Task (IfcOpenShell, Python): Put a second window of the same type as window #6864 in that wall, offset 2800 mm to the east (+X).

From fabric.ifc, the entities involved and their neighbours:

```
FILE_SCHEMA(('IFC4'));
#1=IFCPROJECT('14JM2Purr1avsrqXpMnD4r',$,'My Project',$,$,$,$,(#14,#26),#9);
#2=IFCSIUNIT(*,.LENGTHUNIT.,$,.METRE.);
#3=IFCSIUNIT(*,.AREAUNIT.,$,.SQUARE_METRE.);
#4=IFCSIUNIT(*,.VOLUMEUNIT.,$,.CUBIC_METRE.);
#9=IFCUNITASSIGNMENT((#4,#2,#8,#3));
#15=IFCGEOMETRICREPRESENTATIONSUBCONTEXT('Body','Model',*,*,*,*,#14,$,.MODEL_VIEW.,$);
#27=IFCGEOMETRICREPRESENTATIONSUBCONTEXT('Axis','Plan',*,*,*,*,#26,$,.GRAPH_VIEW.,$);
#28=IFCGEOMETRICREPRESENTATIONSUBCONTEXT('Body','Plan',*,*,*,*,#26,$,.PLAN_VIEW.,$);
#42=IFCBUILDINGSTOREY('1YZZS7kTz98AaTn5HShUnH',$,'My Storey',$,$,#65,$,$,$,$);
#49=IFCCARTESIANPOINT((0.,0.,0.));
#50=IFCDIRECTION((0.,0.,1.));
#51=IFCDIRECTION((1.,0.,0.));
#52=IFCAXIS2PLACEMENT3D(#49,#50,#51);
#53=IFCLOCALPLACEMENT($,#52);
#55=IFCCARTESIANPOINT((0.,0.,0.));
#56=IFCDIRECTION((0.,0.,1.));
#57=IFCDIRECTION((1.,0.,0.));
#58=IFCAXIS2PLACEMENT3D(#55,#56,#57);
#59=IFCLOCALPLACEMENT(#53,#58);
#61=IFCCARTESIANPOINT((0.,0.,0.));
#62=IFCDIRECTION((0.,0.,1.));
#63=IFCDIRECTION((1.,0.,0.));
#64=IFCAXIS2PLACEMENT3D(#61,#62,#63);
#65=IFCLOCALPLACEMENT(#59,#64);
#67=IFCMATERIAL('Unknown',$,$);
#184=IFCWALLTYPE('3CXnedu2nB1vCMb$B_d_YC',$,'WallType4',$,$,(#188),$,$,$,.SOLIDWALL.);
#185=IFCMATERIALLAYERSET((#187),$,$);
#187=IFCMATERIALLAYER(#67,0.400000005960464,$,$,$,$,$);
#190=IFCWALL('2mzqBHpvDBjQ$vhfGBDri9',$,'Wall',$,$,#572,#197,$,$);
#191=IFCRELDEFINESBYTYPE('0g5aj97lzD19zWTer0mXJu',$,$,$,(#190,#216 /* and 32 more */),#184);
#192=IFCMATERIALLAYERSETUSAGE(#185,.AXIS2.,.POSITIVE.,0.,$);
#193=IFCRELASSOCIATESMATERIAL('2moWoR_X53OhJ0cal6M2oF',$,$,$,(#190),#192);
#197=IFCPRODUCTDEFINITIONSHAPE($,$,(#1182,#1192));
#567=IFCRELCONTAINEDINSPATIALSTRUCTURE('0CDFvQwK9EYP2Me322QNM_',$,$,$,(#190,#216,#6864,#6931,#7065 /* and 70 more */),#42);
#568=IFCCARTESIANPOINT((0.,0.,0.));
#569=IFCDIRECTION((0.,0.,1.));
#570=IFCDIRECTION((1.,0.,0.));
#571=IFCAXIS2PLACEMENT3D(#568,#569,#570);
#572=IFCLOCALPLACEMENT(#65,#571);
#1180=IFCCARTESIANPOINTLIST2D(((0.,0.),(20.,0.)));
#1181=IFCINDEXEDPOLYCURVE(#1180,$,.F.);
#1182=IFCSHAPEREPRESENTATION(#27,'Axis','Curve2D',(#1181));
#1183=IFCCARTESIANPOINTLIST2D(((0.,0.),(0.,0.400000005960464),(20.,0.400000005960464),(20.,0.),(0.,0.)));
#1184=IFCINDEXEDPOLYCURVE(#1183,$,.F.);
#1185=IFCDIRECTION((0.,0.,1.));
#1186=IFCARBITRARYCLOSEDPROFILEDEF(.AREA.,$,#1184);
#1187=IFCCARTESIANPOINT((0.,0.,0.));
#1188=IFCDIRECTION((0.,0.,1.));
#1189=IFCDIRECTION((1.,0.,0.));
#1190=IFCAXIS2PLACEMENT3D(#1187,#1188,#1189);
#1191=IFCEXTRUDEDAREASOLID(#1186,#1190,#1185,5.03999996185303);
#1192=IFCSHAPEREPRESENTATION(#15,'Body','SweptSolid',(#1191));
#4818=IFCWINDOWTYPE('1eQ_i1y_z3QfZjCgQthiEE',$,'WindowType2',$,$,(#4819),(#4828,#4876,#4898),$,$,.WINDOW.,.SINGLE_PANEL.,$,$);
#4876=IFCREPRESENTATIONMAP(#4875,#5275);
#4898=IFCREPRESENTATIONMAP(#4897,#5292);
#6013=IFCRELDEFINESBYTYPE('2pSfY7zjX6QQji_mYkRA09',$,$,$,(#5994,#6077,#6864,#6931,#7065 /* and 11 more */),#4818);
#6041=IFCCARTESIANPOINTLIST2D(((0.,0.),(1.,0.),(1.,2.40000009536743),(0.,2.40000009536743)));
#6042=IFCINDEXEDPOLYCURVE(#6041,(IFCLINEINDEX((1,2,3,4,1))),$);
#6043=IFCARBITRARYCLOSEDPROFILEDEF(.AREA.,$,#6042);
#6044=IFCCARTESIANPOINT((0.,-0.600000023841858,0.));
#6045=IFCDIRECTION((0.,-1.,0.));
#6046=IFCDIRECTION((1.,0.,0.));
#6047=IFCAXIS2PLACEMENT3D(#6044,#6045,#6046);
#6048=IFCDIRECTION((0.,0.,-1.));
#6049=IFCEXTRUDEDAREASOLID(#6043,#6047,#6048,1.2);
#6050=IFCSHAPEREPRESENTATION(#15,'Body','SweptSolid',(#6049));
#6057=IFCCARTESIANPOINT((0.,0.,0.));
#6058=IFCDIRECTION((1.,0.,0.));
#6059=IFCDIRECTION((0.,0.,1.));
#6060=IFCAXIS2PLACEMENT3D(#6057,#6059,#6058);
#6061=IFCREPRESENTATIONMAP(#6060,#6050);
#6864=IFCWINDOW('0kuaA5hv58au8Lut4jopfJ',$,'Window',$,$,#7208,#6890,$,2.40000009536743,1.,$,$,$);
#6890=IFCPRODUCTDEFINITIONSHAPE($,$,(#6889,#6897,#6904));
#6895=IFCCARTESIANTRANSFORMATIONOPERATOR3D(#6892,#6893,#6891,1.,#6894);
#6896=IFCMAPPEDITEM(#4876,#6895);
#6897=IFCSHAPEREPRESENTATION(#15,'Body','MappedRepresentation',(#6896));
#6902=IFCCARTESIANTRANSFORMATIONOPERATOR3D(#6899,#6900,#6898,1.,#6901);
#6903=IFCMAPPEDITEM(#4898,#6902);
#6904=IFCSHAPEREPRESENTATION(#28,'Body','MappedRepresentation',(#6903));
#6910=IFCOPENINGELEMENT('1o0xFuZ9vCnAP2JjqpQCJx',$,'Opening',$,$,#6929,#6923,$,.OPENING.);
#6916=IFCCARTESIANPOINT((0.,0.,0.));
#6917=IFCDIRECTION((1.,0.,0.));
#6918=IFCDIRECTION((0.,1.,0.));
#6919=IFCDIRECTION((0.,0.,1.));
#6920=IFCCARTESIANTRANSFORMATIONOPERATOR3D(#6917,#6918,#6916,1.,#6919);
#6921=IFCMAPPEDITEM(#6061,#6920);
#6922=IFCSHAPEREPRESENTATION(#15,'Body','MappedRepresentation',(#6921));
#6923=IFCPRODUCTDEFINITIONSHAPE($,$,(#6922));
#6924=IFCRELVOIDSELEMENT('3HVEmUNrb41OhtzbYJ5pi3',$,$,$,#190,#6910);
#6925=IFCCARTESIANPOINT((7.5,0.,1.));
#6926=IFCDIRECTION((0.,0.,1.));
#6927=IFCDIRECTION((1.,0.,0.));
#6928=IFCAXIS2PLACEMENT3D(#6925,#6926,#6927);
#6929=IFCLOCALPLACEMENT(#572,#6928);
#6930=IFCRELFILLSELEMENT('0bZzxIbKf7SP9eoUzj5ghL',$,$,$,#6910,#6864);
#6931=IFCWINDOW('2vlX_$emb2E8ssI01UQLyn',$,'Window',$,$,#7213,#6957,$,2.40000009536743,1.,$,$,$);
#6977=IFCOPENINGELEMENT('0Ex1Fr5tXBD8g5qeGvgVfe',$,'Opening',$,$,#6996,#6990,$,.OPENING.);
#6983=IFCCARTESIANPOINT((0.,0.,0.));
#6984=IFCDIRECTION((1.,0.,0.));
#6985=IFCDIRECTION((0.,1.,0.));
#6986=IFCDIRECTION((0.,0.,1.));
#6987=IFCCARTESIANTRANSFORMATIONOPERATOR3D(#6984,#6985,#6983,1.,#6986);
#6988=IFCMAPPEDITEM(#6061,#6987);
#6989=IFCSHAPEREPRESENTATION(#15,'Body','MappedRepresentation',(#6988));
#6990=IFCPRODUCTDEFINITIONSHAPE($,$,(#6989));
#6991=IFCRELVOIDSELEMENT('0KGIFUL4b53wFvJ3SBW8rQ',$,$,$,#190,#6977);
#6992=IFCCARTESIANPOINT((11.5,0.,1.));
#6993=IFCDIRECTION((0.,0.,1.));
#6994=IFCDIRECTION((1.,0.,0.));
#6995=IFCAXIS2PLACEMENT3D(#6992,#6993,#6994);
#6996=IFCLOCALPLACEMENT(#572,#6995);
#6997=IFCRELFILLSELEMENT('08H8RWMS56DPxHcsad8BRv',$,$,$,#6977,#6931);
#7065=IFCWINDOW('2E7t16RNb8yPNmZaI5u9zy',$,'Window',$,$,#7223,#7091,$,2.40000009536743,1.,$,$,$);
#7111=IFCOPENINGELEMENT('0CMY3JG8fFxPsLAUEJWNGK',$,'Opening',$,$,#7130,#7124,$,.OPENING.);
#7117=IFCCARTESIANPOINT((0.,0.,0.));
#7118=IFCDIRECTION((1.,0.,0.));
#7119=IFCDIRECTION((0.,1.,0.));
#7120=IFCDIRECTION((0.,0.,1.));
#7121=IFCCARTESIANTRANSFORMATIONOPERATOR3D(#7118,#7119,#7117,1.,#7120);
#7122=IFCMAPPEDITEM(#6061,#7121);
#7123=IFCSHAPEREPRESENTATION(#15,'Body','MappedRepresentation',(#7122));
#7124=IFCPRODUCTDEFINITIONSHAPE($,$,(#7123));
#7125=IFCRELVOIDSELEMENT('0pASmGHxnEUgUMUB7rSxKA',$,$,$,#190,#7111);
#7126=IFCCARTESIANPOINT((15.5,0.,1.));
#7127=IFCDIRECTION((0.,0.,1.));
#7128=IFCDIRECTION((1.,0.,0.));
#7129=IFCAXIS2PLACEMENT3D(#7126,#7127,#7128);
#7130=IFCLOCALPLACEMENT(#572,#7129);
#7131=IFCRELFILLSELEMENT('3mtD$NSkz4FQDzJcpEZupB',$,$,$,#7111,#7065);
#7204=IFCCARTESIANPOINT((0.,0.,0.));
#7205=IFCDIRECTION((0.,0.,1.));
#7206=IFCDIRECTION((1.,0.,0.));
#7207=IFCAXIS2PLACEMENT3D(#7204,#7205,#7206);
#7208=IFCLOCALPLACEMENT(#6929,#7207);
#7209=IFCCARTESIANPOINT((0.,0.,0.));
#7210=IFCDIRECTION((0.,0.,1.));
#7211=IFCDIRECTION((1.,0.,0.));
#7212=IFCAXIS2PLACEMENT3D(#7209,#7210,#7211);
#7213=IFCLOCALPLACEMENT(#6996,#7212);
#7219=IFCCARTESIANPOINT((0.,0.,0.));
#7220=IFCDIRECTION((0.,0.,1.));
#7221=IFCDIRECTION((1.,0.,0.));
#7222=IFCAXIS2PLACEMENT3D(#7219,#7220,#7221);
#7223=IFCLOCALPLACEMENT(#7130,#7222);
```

```python
import ifcopenshell
import ifcopenshell.api.feature
import ifcopenshell.api.geometry
import ifcopenshell.api.root
import ifcopenshell.geom
import ifcopenshell.util.element
import ifcopenshell.util.placement
import ifcopenshell.util.shape
import ifcopenshell.util.unit

model = ifcopenshell.open("fabric.ifc")
unit_scale = ifcopenshell.util.unit.calculate_unit_scale(model)
settings = ifcopenshell.geom.settings()


def volume(element):
    """Net volume in cubic metres, openings subtracted."""
    shape = ifcopenshell.geom.create_shape(settings, element)
    return ifcopenshell.util.shape.get_volume(shape.geometry)


window = model.by_guid("0kuaA5hv58au8Lut4jopfJ")
opening = window.FillsVoids[0].RelatingOpeningElement
wall = opening.VoidsElements[0].RelatingBuildingElement
before = volume(wall)
shift = ifcopenshell.util.placement.get_local_placement(wall.ObjectPlacement)[:3, 0] * 2.8 / unit_scale

# copy_class copies the void relationship, type, container and properties, but no geometry.
new_opening = ifcopenshell.api.root.copy_class(model, product=opening)
new_opening.Representation = ifcopenshell.util.element.copy_deep(
    model, opening.Representation, exclude=["IfcGeometricRepresentationContext", "IfcRepresentationMap"]
)
new_window = ifcopenshell.api.root.copy_class(model, product=window)
new_window.Representation = ifcopenshell.util.element.copy_deep(
    model, window.Representation, exclude=["IfcGeometricRepresentationContext", "IfcRepresentationMap"]
)
ifcopenshell.api.feature.add_filling(model, opening=new_opening, element=new_window)

for old, new in ((opening, new_opening), (window, new_window)):
    matrix = ifcopenshell.util.placement.get_local_placement(old.ObjectPlacement)
    matrix[:3, 3] += shift
    ifcopenshell.api.geometry.edit_object_placement(model, product=new, matrix=matrix, is_si=False)

after = volume(wall)

print(f"wall volume {before:.3f} -> {after:.3f} m3")

model.write("fabric_rev.ifc")
```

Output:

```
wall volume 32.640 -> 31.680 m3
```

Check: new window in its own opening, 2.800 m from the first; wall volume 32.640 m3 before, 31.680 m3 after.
